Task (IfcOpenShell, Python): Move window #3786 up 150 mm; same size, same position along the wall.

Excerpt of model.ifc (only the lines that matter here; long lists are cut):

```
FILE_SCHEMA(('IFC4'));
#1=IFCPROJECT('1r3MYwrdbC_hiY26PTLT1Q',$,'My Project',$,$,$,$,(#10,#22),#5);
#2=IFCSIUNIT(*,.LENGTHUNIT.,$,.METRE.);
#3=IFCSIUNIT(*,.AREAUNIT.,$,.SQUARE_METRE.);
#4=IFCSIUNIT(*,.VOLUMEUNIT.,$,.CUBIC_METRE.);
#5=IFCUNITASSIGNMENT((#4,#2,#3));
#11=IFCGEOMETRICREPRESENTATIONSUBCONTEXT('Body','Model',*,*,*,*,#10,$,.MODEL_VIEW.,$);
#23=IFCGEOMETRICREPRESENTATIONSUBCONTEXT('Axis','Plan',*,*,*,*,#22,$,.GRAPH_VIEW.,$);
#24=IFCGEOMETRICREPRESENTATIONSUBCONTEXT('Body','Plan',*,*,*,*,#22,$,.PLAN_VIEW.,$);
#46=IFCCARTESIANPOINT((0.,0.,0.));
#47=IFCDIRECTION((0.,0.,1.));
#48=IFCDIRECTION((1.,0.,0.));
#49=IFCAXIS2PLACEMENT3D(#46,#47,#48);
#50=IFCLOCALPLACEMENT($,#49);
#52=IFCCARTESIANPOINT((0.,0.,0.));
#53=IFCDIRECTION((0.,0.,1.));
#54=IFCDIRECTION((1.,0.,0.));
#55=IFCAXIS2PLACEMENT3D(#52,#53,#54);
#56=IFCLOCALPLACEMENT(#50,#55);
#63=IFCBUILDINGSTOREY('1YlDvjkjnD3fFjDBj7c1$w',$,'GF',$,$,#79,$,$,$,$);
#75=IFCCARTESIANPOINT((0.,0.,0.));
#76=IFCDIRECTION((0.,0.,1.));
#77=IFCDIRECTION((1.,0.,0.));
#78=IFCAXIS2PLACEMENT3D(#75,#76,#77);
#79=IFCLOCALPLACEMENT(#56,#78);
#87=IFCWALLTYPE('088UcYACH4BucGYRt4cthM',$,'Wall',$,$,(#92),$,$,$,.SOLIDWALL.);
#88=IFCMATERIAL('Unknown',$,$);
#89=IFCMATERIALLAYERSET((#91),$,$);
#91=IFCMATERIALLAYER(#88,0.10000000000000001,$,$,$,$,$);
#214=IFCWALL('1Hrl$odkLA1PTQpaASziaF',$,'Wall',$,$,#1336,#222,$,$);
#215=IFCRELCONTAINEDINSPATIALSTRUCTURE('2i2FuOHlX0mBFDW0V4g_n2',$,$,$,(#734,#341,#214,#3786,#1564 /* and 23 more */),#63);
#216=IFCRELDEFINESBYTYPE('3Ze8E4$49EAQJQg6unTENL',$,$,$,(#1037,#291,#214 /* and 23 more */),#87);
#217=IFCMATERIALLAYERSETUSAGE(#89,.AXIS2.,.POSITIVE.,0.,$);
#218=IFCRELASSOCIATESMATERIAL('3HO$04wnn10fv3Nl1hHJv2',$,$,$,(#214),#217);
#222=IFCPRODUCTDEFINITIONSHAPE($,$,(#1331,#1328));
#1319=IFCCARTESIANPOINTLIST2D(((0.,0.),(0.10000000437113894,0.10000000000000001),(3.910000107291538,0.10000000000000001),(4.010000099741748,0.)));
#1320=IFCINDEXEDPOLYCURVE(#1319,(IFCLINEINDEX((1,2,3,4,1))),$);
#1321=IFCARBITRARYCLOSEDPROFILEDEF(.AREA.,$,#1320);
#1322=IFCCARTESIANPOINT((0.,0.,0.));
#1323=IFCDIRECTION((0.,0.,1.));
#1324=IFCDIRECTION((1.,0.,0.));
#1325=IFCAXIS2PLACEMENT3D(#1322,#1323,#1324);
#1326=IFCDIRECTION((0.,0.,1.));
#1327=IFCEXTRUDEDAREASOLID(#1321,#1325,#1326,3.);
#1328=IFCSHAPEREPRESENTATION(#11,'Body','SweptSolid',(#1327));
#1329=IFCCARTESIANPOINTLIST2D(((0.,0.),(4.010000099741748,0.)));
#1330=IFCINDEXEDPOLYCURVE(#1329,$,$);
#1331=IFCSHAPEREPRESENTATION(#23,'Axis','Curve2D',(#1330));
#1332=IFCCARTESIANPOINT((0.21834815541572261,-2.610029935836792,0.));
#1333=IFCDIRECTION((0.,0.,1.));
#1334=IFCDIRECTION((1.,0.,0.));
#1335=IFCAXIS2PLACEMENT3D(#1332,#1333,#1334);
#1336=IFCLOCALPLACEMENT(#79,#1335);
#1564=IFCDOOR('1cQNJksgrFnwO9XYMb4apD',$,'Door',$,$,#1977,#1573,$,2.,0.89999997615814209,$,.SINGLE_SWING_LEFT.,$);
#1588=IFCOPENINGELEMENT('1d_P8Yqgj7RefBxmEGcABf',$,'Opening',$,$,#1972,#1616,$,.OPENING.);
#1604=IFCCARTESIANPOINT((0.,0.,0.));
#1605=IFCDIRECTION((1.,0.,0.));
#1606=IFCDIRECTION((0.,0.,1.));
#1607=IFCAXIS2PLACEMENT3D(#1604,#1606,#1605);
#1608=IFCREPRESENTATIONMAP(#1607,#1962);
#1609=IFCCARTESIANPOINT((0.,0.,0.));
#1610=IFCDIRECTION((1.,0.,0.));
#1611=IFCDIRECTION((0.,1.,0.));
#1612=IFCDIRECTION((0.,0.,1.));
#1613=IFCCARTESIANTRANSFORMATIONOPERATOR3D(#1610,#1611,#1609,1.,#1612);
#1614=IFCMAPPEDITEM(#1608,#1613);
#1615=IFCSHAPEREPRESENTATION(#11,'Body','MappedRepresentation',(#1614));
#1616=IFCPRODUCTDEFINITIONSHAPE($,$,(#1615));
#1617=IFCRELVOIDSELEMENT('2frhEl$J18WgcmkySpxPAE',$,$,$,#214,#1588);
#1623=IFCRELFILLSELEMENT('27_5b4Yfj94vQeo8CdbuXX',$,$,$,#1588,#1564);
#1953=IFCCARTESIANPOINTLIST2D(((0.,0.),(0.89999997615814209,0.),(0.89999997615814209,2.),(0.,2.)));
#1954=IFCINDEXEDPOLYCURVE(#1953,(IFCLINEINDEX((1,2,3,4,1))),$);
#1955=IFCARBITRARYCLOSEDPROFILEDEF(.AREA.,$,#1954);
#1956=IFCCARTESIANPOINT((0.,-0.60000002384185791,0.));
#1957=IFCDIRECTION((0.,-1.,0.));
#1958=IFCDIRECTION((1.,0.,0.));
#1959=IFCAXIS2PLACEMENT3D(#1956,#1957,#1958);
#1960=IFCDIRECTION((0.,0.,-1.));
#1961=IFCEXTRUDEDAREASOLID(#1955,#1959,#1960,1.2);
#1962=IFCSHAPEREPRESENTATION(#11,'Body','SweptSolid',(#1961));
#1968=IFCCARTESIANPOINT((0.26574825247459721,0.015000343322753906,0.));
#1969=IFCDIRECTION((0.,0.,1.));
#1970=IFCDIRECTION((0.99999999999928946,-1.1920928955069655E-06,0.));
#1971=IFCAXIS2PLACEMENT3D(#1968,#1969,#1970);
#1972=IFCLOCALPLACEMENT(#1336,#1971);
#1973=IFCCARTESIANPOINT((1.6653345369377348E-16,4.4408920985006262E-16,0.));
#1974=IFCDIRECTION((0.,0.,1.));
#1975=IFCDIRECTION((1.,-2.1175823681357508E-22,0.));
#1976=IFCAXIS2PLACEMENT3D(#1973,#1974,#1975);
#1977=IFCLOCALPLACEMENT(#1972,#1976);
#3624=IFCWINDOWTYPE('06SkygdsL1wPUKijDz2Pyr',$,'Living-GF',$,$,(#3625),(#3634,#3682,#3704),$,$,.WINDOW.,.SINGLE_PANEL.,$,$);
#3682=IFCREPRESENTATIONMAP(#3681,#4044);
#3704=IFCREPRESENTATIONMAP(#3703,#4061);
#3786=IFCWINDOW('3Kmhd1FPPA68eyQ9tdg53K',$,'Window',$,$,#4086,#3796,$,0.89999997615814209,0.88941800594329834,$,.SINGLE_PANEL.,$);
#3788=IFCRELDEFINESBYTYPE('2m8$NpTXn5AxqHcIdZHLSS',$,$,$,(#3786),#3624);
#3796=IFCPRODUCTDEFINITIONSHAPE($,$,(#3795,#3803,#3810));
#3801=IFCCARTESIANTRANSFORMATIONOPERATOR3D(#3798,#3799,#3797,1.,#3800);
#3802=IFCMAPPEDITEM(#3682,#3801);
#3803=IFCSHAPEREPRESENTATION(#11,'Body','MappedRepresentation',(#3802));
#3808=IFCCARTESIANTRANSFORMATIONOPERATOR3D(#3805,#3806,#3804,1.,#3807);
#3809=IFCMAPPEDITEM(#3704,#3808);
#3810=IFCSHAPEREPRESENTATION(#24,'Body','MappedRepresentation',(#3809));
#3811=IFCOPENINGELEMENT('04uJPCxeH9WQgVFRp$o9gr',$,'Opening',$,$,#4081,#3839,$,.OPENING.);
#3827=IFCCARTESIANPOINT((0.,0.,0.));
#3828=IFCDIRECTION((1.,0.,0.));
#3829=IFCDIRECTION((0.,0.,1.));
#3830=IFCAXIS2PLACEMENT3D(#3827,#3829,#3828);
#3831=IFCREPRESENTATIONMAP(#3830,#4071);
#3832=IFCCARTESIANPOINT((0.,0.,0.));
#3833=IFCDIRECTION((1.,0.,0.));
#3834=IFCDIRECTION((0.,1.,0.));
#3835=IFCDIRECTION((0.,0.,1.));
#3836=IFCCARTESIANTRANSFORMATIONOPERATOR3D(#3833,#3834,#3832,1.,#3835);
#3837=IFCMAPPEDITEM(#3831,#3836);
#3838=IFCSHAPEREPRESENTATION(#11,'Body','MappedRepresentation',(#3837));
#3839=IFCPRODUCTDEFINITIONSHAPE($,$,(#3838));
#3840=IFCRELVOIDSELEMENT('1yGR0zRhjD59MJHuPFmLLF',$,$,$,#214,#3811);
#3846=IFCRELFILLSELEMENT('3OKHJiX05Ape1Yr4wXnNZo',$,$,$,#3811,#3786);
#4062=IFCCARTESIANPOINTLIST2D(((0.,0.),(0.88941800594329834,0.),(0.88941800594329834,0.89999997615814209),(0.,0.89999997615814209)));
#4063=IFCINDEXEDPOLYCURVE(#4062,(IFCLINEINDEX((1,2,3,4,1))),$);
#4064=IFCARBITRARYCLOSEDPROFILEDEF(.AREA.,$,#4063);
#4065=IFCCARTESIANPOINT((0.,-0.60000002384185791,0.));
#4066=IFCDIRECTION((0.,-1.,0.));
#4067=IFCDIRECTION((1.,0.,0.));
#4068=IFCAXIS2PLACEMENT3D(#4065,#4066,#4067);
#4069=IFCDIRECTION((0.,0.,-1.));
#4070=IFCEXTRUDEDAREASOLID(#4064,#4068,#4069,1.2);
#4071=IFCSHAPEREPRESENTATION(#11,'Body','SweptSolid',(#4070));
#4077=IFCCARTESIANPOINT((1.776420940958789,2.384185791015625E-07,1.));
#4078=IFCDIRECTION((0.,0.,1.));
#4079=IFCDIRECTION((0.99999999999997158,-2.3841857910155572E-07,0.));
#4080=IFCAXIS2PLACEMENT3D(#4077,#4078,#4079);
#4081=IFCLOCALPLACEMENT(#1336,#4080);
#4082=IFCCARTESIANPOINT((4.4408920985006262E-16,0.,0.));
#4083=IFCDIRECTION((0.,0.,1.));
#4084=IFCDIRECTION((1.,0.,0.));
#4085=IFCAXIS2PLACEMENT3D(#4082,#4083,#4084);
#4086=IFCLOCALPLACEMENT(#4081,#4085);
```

```python
import numpy as np
import ifcopenshell
import ifcopenshell.api.geometry
import ifcopenshell.util.placement
import ifcopenshell.util.unit

model = ifcopenshell.open("model.ifc")
unit_scale = ifcopenshell.util.unit.calculate_unit_scale(model)

window = model.by_id(3786)
opening = window.FillsVoids[0].RelatingOpeningElement
dz = 0.15 / unit_scale

shift = np.array([0.0, 0.0, dz])
# The window is placed relative to its opening, so it follows when the opening moves.
matrix = ifcopenshell.util.placement.get_local_placement(opening.ObjectPlacement)
matrix[:3, 3] += shift
ifcopenshell.api.geometry.edit_object_placement(
    model, product=opening, matrix=matrix, is_si=False, should_transform_children=True
)

print(f"moved by {dz * unit_scale:+.3f} m")

model.write("model-out.ifc")
```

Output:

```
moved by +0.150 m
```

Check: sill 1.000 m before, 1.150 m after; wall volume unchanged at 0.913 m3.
